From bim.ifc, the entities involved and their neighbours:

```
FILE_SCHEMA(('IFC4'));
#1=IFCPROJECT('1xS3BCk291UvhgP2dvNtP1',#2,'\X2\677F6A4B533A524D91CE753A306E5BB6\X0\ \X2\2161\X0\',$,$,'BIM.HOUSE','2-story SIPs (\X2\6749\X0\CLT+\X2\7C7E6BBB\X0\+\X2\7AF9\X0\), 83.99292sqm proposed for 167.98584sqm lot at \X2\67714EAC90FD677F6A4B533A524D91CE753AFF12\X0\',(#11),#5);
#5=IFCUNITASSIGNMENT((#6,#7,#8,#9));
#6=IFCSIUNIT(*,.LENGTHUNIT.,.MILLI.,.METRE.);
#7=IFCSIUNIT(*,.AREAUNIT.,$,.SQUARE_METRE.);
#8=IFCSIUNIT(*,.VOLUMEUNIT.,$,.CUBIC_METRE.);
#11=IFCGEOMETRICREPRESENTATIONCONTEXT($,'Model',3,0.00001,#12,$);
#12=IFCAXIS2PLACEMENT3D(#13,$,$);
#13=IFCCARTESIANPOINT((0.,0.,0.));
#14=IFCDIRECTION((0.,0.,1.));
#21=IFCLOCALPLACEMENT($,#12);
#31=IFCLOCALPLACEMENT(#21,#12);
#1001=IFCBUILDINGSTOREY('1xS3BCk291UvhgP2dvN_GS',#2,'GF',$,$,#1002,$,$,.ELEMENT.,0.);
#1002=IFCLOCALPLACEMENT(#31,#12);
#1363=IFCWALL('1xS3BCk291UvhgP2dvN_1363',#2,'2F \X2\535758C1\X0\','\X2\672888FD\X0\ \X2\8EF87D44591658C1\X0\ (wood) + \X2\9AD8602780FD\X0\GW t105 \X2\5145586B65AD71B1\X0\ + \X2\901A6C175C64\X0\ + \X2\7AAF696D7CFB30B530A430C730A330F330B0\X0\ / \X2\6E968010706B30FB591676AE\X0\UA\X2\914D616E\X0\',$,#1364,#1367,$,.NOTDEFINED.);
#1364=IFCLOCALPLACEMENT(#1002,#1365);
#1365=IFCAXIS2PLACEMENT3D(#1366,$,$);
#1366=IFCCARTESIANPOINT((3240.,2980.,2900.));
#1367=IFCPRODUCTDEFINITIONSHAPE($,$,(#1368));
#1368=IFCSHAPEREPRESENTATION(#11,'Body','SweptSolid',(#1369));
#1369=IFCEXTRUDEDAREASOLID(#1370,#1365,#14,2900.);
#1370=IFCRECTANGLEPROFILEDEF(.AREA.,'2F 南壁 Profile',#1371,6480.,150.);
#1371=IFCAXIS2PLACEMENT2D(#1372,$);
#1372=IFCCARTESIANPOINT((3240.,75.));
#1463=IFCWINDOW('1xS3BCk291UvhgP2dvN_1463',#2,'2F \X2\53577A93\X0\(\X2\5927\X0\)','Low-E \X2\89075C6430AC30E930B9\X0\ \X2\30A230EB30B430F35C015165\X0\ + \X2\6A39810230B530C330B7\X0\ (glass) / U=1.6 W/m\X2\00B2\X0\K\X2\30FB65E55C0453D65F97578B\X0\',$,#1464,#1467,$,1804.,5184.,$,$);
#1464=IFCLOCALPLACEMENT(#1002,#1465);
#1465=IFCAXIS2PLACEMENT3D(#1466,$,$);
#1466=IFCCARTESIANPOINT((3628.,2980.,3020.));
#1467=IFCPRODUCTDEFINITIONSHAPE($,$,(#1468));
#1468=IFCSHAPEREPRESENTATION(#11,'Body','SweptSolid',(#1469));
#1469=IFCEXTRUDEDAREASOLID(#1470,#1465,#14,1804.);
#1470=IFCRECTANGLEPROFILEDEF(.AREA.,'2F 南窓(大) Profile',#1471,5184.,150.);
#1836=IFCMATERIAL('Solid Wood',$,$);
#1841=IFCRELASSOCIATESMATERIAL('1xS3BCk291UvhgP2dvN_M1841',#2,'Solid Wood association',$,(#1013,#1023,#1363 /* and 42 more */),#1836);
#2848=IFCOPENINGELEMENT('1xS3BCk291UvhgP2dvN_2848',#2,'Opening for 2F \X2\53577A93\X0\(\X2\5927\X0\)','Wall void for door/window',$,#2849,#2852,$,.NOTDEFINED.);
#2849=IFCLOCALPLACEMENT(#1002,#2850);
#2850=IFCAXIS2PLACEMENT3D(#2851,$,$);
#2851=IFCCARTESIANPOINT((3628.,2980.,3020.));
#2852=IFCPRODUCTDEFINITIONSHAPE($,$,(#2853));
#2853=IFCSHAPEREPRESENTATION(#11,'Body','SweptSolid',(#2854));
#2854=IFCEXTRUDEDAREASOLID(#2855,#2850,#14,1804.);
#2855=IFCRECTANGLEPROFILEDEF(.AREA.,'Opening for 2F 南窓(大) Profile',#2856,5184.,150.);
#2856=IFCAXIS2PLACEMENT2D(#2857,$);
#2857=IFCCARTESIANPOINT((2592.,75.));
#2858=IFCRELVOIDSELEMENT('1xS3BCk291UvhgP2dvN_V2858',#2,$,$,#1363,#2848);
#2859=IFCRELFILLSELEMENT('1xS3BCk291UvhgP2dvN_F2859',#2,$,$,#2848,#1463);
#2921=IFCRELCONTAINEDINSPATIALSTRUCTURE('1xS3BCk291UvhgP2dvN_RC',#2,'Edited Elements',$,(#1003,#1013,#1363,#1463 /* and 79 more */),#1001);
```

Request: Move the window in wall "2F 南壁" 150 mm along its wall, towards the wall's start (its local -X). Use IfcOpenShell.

```python
import ifcopenshell
import ifcopenshell.api.geometry
import ifcopenshell.util.placement
import ifcopenshell.util.unit

model = ifcopenshell.open("bim.ifc")
unit_scale = ifcopenshell.util.unit.calculate_unit_scale(model)

window = model.by_id(1463)
opening = window.FillsVoids[0].RelatingOpeningElement
wall = opening.VoidsElements[0].RelatingBuildingElement

wall_matrix = ifcopenshell.util.placement.get_local_placement(wall.ObjectPlacement)
shift = wall_matrix[:3, 0] * -0.15 / unit_scale
before = ifcopenshell.util.placement.get_local_placement(window.ObjectPlacement)[:3, 3].copy()

# The window is not placed relative to its opening, so move both.
for product in (opening, window):
    matrix = ifcopenshell.util.placement.get_local_placement(product.ObjectPlacement)
    matrix[:3, 3] += shift
    ifcopenshell.api.geometry.edit_object_placement(model, product=product, matrix=matrix, is_si=False)

after = ifcopenshell.util.placement.get_local_placement(window.ObjectPlacement)[:3, 3]
print("window moved by", (after - before).round(3) + 0.0)

model.write("bim_v2.ifc")
```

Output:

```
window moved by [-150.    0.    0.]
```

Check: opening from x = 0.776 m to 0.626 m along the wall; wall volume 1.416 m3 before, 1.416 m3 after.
